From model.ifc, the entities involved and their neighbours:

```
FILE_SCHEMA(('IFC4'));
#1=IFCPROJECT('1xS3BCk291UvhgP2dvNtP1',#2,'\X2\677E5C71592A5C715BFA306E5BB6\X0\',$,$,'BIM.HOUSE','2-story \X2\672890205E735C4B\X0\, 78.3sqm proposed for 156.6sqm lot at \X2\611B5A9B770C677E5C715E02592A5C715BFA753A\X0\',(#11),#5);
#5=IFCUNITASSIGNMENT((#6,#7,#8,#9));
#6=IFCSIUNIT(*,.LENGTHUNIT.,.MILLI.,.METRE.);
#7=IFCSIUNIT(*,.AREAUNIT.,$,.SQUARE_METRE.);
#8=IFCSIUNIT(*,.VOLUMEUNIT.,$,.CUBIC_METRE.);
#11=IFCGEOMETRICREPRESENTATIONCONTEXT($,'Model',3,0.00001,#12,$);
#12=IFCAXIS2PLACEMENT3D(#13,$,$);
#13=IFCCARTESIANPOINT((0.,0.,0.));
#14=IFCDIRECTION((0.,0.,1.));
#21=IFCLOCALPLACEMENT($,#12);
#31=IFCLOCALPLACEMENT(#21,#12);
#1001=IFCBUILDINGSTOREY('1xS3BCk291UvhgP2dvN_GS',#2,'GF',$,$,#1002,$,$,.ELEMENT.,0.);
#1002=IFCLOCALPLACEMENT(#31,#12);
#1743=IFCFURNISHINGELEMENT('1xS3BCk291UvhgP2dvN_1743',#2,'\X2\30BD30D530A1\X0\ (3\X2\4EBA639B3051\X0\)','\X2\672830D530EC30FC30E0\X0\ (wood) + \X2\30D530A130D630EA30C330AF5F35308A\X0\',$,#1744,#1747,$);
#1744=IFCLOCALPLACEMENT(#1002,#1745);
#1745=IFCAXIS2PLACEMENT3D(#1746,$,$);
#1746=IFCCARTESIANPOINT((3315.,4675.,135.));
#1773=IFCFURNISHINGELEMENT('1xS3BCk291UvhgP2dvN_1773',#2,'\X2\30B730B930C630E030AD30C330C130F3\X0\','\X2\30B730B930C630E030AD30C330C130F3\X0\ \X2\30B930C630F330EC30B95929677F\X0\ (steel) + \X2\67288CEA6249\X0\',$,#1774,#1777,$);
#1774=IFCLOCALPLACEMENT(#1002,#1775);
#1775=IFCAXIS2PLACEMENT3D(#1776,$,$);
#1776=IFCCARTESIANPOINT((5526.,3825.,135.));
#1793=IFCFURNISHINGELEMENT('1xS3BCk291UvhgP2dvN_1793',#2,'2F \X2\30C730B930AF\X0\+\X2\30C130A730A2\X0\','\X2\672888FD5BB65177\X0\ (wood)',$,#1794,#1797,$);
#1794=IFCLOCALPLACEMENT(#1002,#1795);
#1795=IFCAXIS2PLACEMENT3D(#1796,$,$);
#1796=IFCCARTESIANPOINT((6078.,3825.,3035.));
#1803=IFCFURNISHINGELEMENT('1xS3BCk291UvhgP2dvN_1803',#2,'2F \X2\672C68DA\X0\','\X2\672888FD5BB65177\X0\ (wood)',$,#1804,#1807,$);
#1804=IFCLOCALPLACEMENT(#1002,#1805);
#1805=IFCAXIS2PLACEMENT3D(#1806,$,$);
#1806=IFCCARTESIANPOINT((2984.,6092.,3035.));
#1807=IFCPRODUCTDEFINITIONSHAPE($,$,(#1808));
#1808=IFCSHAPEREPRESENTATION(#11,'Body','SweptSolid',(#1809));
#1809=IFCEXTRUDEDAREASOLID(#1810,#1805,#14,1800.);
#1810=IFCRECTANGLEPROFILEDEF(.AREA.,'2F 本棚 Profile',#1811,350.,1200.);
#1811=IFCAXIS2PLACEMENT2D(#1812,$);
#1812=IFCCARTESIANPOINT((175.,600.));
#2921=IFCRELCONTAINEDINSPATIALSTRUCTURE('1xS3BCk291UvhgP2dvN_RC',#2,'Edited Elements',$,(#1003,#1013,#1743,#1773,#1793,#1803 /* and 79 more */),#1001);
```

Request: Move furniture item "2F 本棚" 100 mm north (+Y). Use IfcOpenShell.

```python
import ifcopenshell
import ifcopenshell.api.geometry
import ifcopenshell.util.placement

model = ifcopenshell.open("model.ifc")

item = model.by_id(1803)
matrix = ifcopenshell.util.placement.get_local_placement(item.ObjectPlacement)
matrix[1, 3] += 100.0
ifcopenshell.api.geometry.edit_object_placement(model, product=item, matrix=matrix, is_si=False)

print(ifcopenshell.util.placement.get_local_placement(item.ObjectPlacement).round(3) + 0.0)

model.write("model_updated.ifc")
```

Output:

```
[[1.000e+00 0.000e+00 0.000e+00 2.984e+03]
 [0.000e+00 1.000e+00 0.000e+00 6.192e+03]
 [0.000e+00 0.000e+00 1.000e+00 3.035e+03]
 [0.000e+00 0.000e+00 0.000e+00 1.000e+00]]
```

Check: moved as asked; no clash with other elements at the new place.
